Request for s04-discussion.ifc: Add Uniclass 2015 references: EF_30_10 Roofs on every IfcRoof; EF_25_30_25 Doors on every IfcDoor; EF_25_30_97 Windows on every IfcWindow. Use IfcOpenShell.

First a look at what the model holds.

```python
import ifcopenshell

model = ifcopenshell.open("s04-discussion.ifc")
print(model.schema)
print("classifications:", [c.Name for c in model.by_type("IfcClassification")])
for ifc_class in ("IfcDoor", "IfcRoof", "IfcStair", "IfcWall", "IfcWindow"):
    print(ifc_class, len(model.by_type(ifc_class)))
```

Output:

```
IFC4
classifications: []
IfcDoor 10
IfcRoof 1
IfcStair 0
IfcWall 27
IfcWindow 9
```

```python
import ifcopenshell
import ifcopenshell.api.classification

model = ifcopenshell.open("s04-discussion.ifc")

system = ifcopenshell.api.classification.add_classification(model, classification="Uniclass 2015")

codes = {
    "IfcRoof": ("EF_30_10", "Roofs"),
    "IfcDoor": ("EF_25_30_25", "Doors"),
    "IfcWindow": ("EF_25_30_97", "Windows"),
}
for ifc_class, (code, name) in codes.items():
    products = model.by_type(ifc_class)
    ifcopenshell.api.classification.add_reference(
        model, products=products, classification=system, identification=code, name=name
    )
    print(code, len(products))

model.write("s04-discussion_rev.ifc")
```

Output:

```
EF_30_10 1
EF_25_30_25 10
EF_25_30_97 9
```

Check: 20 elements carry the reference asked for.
